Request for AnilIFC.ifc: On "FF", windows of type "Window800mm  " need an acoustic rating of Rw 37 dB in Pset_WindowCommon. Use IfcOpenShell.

First a look at what the model holds.

```python
import ifcopenshell
import ifcopenshell.util.element

model = ifcopenshell.open("AnilIFC.ifc")
print(model.schema)
storey = next(s for s in model.by_type("IfcBuildingStorey") if s.Name == "FF")
windows = [e for e in ifcopenshell.util.element.get_decomposition(storey) if e.is_a("IfcWindow")]
seen = {}
for e in windows:
    element_type = ifcopenshell.util.element.get_type(e)
    key = (element_type.Name if element_type != e and element_type else None, ifcopenshell.util.element.get_pset(e, "Pset_WindowCommon", "AcousticRating"))
    seen[key] = seen.get(key, 0) + 1
for (name, value), count in sorted(seen.items(), key=str):
    print(count, "x", name, "|", value)
```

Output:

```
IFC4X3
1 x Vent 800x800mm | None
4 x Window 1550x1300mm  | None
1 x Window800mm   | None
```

```python
import ifcopenshell
import ifcopenshell.api.pset
import ifcopenshell.util.element

model = ifcopenshell.open("AnilIFC.ifc")

storey = next(s for s in model.by_type("IfcBuildingStorey") if s.Name == "FF")
windows = [e for e in ifcopenshell.util.element.get_decomposition(storey) if e.is_a("IfcWindow")]

count = 0
for e in windows:
    element_type = ifcopenshell.util.element.get_type(e)
    if element_type in (None, e) or element_type.Name != "Window800mm  ":
        continue
    # add_pset returns the element's existing set when there is one.
    pset = ifcopenshell.api.pset.add_pset(model, product=e, name="Pset_WindowCommon")
    ifcopenshell.api.pset.edit_pset(model, pset=pset, properties={"AcousticRating": "Rw 37 dB"})
    count += 1

print(count, "windows updated")

model.write("AnilIFC_updated.ifc")
```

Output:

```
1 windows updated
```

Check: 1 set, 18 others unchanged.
